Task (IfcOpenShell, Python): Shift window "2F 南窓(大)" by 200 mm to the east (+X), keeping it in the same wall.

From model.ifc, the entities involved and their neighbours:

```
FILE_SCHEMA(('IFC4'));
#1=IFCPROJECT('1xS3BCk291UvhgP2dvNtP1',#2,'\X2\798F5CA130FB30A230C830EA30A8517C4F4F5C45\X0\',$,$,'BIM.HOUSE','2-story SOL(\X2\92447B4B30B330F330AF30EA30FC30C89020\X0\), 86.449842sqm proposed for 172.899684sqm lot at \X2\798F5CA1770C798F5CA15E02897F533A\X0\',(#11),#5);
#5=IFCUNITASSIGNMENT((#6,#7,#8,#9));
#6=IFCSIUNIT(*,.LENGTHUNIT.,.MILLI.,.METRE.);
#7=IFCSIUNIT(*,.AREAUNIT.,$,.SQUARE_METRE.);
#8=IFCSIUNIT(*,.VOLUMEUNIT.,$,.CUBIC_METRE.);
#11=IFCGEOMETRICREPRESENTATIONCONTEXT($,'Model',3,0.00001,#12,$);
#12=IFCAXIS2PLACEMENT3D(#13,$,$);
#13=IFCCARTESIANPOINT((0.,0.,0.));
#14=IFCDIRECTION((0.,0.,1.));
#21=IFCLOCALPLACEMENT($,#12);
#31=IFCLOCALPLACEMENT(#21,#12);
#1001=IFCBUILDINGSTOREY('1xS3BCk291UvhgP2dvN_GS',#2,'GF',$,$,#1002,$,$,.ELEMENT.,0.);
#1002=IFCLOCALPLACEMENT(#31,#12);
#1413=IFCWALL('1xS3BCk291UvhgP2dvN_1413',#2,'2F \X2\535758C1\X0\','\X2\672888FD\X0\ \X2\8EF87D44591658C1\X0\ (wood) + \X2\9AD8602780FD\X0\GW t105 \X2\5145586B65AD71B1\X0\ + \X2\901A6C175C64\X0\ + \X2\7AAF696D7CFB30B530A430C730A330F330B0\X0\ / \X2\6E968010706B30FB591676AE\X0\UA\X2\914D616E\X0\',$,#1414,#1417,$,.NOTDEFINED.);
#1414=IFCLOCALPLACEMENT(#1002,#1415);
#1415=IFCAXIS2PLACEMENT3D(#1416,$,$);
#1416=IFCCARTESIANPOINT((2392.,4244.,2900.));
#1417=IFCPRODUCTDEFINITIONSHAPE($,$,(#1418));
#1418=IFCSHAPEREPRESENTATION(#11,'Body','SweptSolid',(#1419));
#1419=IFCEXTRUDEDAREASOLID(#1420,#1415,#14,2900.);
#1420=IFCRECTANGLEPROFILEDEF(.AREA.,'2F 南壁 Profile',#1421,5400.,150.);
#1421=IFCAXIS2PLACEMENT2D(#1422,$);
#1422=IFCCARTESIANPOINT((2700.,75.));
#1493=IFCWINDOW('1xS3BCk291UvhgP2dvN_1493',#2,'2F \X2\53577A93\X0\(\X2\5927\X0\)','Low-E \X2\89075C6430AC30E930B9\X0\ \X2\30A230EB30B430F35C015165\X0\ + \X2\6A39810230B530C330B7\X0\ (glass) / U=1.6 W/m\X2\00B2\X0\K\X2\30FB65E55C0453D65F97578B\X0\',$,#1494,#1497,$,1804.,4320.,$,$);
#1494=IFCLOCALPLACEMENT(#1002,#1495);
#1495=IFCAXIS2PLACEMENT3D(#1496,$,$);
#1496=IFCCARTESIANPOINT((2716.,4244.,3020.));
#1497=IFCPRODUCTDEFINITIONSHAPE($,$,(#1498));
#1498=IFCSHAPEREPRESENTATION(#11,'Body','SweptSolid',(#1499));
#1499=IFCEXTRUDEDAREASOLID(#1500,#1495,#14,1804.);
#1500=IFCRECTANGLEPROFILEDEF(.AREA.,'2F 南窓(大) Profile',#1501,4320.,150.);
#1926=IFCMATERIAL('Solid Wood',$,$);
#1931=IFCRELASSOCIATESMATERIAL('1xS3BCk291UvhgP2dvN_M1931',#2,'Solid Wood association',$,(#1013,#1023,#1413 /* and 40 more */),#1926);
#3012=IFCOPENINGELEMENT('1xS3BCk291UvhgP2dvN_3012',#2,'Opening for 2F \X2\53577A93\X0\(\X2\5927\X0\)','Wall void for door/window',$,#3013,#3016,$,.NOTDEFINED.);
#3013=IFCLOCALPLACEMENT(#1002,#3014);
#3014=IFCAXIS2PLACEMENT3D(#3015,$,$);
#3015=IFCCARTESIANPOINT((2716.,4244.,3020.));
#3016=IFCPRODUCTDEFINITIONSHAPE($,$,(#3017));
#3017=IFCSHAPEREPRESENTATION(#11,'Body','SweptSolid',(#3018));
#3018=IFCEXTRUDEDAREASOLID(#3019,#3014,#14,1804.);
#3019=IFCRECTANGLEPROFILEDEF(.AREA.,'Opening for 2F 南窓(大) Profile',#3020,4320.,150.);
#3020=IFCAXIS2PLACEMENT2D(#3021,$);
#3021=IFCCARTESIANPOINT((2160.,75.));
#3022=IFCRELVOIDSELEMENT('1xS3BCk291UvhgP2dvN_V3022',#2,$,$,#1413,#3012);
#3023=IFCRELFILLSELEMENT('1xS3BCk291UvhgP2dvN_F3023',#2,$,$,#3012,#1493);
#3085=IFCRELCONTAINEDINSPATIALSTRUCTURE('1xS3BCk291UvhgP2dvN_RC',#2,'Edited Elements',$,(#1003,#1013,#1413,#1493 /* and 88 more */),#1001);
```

```python
import ifcopenshell
import ifcopenshell.api.geometry
import ifcopenshell.util.placement

model = ifcopenshell.open("model.ifc")

window = model.by_guid("1xS3BCk291UvhgP2dvN_1493")
opening = window.FillsVoids[0].RelatingOpeningElement
wall = opening.VoidsElements[0].RelatingBuildingElement

wall_matrix = ifcopenshell.util.placement.get_local_placement(wall.ObjectPlacement)
shift = wall_matrix[:3, 0] * 200.0
before = ifcopenshell.util.placement.get_local_placement(window.ObjectPlacement)[:3, 3].copy()

# The window is not placed relative to its opening, so move both.
for product in (opening, window):
    matrix = ifcopenshell.util.placement.get_local_placement(product.ObjectPlacement)
    matrix[:3, 3] += shift
    ifcopenshell.api.geometry.edit_object_placement(model, product=product, matrix=matrix, is_si=False)

after = ifcopenshell.util.placement.get_local_placement(window.ObjectPlacement)[:3, 3]
print("window moved by", (after - before).round(3) + 0.0)

model.write("model_edited.ifc")
```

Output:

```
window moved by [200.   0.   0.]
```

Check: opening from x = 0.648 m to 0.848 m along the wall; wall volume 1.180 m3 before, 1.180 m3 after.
